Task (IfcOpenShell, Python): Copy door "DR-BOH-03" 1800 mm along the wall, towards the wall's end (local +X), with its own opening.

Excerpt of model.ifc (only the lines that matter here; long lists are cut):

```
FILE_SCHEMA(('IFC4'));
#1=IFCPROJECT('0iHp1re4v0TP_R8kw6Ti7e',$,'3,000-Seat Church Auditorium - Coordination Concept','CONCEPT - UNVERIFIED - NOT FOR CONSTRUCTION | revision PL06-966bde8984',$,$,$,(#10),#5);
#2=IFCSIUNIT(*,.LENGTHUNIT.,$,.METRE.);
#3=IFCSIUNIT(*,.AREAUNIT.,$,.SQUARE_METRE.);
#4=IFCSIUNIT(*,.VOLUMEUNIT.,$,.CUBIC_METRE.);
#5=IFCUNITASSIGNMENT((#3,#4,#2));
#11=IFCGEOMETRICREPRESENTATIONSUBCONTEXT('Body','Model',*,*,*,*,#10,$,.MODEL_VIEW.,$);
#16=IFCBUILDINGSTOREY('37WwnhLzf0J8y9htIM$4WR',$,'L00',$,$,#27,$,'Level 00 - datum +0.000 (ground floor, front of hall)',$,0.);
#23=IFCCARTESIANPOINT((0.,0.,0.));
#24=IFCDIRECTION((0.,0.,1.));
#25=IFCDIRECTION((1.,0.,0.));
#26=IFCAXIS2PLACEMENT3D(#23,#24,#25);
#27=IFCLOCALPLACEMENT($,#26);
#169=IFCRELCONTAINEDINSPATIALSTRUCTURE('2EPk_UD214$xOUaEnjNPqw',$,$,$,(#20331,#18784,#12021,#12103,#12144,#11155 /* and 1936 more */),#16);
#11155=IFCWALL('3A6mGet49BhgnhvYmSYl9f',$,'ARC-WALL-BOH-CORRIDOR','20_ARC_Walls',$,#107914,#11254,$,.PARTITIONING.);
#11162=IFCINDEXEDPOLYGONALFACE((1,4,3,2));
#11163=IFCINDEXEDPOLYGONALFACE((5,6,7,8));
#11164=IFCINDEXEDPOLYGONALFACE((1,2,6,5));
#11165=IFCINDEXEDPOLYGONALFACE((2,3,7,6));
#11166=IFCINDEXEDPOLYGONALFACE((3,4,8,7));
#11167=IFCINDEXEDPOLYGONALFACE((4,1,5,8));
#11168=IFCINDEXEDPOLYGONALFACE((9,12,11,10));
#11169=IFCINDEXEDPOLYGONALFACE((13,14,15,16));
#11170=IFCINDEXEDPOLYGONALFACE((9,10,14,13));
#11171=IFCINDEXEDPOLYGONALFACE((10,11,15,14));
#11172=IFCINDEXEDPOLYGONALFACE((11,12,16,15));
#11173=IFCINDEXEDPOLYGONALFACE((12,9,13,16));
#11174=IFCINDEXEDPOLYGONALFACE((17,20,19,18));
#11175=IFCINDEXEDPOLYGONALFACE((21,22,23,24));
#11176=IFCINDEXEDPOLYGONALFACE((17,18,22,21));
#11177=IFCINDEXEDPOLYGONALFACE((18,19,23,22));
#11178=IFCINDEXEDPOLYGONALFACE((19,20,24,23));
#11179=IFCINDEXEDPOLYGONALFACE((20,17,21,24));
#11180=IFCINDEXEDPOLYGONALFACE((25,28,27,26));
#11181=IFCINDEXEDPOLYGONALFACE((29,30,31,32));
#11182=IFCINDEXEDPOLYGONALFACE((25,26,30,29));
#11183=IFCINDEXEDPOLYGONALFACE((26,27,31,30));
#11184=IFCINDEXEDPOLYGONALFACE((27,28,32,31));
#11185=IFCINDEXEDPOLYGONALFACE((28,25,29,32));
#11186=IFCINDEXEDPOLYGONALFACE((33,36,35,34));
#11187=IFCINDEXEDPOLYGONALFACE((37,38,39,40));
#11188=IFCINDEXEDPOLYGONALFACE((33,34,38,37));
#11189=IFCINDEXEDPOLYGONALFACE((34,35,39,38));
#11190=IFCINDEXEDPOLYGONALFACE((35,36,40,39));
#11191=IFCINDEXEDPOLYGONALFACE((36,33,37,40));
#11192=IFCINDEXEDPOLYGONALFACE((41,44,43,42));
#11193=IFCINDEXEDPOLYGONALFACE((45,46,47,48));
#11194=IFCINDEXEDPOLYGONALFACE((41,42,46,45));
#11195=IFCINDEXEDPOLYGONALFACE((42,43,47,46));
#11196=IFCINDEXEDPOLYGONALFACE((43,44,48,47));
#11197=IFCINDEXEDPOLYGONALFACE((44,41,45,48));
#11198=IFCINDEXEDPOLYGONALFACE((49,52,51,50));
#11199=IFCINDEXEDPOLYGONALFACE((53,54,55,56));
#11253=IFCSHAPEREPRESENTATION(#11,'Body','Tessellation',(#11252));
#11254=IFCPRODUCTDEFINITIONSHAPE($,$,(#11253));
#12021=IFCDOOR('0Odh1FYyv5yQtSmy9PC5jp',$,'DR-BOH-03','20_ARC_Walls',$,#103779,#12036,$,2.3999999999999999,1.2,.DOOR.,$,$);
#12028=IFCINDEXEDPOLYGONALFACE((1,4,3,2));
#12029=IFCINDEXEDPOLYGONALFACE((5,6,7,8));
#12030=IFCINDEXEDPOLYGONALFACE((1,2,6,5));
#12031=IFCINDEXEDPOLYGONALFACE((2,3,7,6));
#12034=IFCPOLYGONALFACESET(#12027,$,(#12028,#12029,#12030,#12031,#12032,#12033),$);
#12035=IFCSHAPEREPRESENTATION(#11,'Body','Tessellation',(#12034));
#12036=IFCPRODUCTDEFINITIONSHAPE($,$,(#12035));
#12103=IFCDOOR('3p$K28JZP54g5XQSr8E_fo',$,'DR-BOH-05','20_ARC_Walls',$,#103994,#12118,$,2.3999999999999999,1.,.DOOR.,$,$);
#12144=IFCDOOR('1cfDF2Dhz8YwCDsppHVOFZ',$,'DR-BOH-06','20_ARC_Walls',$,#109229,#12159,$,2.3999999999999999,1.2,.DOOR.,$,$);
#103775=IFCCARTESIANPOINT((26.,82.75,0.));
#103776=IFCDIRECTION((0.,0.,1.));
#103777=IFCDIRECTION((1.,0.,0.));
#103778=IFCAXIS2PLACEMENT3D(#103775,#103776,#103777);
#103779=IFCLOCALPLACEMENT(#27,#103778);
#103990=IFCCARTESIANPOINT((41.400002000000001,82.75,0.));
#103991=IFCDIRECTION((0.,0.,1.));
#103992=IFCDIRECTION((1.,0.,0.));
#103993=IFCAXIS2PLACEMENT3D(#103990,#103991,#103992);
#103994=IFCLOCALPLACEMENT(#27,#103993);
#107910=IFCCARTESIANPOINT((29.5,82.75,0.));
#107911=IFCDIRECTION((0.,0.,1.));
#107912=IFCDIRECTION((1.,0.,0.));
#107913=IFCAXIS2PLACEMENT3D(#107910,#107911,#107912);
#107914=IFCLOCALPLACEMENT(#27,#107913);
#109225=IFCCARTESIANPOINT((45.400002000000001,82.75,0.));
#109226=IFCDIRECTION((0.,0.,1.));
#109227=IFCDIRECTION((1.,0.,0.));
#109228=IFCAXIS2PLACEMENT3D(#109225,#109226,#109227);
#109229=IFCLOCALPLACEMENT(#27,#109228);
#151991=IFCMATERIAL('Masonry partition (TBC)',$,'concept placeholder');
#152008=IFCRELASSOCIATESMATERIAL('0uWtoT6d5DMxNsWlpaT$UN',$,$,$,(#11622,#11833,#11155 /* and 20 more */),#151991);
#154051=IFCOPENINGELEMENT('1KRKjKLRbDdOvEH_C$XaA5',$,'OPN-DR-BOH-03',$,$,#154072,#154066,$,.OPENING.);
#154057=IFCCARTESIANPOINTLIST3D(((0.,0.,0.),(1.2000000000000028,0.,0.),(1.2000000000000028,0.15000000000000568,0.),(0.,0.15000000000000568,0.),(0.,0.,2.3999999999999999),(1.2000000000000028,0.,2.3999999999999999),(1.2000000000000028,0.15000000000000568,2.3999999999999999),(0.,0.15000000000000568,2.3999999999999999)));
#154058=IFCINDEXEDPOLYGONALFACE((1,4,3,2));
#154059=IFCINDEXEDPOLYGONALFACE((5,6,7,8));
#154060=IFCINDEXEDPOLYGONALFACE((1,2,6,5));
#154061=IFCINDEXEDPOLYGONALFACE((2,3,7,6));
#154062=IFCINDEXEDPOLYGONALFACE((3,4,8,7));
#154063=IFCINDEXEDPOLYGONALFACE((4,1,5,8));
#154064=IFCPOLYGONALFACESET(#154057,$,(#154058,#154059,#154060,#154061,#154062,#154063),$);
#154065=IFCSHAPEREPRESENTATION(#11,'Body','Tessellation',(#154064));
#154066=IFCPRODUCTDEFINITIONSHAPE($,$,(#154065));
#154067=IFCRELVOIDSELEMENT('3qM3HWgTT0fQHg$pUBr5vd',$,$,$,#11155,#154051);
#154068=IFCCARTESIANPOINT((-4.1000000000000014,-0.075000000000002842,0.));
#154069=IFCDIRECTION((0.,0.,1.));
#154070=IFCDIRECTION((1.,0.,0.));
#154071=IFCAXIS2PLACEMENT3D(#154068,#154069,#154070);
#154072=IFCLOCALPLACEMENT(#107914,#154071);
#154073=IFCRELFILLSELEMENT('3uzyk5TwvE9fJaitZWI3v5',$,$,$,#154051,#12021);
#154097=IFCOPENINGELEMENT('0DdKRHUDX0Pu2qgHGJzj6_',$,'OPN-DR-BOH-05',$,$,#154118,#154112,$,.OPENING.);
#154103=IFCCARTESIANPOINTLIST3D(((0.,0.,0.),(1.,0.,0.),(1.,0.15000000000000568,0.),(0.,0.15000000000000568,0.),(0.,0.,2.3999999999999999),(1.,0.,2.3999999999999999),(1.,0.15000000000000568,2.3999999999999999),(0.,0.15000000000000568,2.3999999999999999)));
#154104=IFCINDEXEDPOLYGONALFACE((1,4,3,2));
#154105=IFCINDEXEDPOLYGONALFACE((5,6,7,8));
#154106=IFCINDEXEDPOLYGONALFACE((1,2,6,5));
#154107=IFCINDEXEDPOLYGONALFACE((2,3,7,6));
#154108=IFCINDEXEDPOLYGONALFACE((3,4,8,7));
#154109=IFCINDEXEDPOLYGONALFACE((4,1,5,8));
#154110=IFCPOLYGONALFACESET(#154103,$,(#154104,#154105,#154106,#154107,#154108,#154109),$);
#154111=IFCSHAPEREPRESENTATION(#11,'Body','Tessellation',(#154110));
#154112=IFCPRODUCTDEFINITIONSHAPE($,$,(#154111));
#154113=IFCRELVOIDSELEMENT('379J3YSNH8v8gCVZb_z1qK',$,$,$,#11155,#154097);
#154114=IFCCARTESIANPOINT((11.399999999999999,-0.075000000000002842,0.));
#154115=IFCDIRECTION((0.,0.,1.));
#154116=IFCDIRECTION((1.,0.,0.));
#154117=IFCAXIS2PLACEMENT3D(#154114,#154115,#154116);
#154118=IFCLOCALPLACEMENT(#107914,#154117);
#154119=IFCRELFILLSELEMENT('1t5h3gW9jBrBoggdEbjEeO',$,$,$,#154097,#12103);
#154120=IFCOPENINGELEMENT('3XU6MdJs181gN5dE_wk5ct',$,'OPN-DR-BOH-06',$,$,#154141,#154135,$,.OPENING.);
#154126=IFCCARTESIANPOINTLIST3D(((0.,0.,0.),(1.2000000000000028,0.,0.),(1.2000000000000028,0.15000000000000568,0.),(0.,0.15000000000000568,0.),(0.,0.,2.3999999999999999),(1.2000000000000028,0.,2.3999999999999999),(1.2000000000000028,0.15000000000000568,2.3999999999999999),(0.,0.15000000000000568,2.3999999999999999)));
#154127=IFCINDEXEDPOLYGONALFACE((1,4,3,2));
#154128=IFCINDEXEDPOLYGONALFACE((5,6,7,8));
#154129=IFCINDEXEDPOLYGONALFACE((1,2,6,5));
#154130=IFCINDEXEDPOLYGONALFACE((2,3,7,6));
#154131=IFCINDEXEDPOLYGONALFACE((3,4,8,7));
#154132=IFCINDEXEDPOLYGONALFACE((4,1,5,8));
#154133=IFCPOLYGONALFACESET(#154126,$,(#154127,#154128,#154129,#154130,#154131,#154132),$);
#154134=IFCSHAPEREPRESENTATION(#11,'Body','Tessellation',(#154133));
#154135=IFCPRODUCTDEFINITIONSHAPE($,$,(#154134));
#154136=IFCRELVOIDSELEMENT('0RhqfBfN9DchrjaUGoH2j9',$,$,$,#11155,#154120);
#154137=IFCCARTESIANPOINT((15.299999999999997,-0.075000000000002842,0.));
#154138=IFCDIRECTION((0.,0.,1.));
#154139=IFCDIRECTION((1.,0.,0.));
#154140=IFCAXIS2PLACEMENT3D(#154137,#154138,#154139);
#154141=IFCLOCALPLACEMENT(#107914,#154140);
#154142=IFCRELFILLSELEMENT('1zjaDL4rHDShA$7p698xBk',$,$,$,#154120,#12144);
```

```python
import ifcopenshell
import ifcopenshell.api.feature
import ifcopenshell.api.geometry
import ifcopenshell.api.root
import ifcopenshell.geom
import ifcopenshell.util.element
import ifcopenshell.util.placement
import ifcopenshell.util.shape

model = ifcopenshell.open("model.ifc")
settings = ifcopenshell.geom.settings()


def volume(element):
    """Net volume in cubic metres, openings subtracted."""
    shape = ifcopenshell.geom.create_shape(settings, element)
    return ifcopenshell.util.shape.get_volume(shape.geometry)


door = model.by_guid("0Odh1FYyv5yQtSmy9PC5jp")
opening = door.FillsVoids[0].RelatingOpeningElement
wall = opening.VoidsElements[0].RelatingBuildingElement
before = volume(wall)
shift = ifcopenshell.util.placement.get_local_placement(wall.ObjectPlacement)[:3, 0] * 1.8

# copy_class copies the void relationship, type, container and properties, but no geometry.
new_opening = ifcopenshell.api.root.copy_class(model, product=opening)
new_opening.Representation = ifcopenshell.util.element.copy_deep(
    model, opening.Representation, exclude=["IfcGeometricRepresentationContext", "IfcRepresentationMap"]
)
new_door = ifcopenshell.api.root.copy_class(model, product=door)
new_door.Representation = ifcopenshell.util.element.copy_deep(
    model, door.Representation, exclude=["IfcGeometricRepresentationContext", "IfcRepresentationMap"]
)
ifcopenshell.api.feature.add_filling(model, opening=new_opening, element=new_door)

for old, new in ((opening, new_opening), (door, new_door)):
    matrix = ifcopenshell.util.placement.get_local_placement(old.ObjectPlacement)
    matrix[:3, 3] += shift
    ifcopenshell.api.geometry.edit_object_placement(model, product=new, matrix=matrix, is_si=False)

after = volume(wall)

print(f"wall volume {before:.3f} -> {after:.3f} m3")

model.write("model_rev.ifc")
```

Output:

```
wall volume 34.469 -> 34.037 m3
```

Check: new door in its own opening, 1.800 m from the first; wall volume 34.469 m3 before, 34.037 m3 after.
